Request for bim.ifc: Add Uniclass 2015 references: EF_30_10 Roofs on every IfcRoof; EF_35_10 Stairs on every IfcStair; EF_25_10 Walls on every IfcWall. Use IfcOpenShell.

First a look at what the model holds.

```python
import ifcopenshell

model = ifcopenshell.open("bim.ifc")
print(model.schema)
print("classifications:", [c.Name for c in model.by_type("IfcClassification")])
for ifc_class in ("IfcDoor", "IfcRoof", "IfcStair", "IfcWall", "IfcWindow"):
    print(ifc_class, len(model.by_type(ifc_class)))
```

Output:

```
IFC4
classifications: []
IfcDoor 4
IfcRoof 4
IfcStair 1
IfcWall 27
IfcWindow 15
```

```python
import ifcopenshell
import ifcopenshell.api.classification

model = ifcopenshell.open("bim.ifc")

system = ifcopenshell.api.classification.add_classification(model, classification="Uniclass 2015")

codes = {
    "IfcRoof": ("EF_30_10", "Roofs"),
    "IfcStair": ("EF_35_10", "Stairs"),
    "IfcWall": ("EF_25_10", "Walls"),
}
for ifc_class, (code, name) in codes.items():
    products = model.by_type(ifc_class)
    ifcopenshell.api.classification.add_reference(
        model, products=products, classification=system, identification=code, name=name
    )
    print(code, len(products))

model.write("bim_edited.ifc")
```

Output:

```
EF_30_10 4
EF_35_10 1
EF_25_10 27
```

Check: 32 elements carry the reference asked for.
